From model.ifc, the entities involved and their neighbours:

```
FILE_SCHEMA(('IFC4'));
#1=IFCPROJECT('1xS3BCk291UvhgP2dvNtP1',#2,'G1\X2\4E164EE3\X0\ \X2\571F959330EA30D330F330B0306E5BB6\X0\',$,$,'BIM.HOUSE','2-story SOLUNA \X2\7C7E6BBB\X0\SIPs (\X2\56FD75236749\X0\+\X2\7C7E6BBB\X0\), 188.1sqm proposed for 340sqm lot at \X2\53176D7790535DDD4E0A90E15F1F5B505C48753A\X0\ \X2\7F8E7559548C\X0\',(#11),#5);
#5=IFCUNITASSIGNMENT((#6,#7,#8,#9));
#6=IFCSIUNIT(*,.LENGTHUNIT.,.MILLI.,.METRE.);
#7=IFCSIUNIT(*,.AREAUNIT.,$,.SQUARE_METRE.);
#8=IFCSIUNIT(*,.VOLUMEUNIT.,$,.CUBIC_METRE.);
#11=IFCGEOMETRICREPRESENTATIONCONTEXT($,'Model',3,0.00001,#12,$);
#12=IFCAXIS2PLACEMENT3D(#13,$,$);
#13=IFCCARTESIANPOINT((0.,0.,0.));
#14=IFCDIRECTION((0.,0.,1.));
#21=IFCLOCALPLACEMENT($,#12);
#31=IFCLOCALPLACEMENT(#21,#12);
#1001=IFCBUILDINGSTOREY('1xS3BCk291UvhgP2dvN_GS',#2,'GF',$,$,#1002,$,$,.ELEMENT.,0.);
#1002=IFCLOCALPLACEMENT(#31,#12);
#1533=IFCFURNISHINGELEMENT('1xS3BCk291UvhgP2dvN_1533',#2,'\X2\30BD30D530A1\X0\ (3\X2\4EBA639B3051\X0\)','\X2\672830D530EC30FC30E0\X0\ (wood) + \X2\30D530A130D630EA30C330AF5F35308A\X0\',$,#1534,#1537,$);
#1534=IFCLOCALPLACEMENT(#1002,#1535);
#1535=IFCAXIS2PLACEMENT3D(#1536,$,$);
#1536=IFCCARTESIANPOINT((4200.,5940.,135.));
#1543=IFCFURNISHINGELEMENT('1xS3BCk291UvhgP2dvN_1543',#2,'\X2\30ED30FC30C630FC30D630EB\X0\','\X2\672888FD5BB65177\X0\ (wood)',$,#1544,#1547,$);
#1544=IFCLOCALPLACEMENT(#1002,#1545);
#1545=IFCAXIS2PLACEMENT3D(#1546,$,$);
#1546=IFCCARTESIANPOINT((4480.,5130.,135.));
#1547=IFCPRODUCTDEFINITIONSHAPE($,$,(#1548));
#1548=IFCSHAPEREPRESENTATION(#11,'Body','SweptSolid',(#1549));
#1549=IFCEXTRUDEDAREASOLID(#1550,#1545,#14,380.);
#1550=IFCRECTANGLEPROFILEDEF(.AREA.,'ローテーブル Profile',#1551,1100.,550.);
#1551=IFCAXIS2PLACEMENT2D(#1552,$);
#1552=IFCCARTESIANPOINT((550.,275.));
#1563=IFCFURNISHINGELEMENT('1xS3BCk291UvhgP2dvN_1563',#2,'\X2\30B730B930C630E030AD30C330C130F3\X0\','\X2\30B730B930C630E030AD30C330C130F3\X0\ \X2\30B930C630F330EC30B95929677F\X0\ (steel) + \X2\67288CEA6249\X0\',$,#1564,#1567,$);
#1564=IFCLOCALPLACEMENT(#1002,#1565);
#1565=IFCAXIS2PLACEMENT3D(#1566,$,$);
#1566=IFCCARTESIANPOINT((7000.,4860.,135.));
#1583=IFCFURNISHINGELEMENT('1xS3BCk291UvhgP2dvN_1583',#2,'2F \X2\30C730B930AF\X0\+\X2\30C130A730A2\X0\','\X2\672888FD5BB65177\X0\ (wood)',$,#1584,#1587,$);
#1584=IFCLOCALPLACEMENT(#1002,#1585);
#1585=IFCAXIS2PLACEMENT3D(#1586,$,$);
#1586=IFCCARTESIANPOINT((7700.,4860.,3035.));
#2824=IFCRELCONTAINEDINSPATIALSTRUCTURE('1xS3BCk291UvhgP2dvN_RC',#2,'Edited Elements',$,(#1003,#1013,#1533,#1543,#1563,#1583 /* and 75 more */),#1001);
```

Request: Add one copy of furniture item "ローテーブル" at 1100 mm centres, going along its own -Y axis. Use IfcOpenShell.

```python
import ifcopenshell
import ifcopenshell.api.geometry
import ifcopenshell.api.root
import ifcopenshell.util.element
import ifcopenshell.util.placement
import ifcopenshell.util.unit

model = ifcopenshell.open("model.ifc")
unit_scale = ifcopenshell.util.unit.calculate_unit_scale(model)


def reuse_history(source, copy):
    """copy_class also copies each property set's owner history, people and application; keep the originals."""
    for rel in copy.IsDefinedBy:
        if rel.is_a("IfcRelDefinesByProperties") and (history := rel.RelatingPropertyDefinition.OwnerHistory):
            rel.RelatingPropertyDefinition.OwnerHistory = source.OwnerHistory
            ifcopenshell.util.element.remove_deep2(model, history)


source = model.by_guid("1xS3BCk291UvhgP2dvN_1543")
base = ifcopenshell.util.placement.get_local_placement(source.ObjectPlacement)
step = -base[:3, 1] * 1.1 / unit_scale

for i in range(1, 2):
    copy = ifcopenshell.api.root.copy_class(model, product=source)
    copy.Representation = ifcopenshell.util.element.copy_deep(
        model, source.Representation, exclude=["IfcGeometricRepresentationContext", "IfcRepresentationMap"]
    )
    reuse_history(source, copy)
    matrix = base.copy()
    matrix[:3, 3] += i * step
    print("added at", matrix[:3, 3].round(3) + 0.0)
    ifcopenshell.api.geometry.edit_object_placement(model, product=copy, matrix=matrix, is_si=False)

model.write("model_updated.ifc")
```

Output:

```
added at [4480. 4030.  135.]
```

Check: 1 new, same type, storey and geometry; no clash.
